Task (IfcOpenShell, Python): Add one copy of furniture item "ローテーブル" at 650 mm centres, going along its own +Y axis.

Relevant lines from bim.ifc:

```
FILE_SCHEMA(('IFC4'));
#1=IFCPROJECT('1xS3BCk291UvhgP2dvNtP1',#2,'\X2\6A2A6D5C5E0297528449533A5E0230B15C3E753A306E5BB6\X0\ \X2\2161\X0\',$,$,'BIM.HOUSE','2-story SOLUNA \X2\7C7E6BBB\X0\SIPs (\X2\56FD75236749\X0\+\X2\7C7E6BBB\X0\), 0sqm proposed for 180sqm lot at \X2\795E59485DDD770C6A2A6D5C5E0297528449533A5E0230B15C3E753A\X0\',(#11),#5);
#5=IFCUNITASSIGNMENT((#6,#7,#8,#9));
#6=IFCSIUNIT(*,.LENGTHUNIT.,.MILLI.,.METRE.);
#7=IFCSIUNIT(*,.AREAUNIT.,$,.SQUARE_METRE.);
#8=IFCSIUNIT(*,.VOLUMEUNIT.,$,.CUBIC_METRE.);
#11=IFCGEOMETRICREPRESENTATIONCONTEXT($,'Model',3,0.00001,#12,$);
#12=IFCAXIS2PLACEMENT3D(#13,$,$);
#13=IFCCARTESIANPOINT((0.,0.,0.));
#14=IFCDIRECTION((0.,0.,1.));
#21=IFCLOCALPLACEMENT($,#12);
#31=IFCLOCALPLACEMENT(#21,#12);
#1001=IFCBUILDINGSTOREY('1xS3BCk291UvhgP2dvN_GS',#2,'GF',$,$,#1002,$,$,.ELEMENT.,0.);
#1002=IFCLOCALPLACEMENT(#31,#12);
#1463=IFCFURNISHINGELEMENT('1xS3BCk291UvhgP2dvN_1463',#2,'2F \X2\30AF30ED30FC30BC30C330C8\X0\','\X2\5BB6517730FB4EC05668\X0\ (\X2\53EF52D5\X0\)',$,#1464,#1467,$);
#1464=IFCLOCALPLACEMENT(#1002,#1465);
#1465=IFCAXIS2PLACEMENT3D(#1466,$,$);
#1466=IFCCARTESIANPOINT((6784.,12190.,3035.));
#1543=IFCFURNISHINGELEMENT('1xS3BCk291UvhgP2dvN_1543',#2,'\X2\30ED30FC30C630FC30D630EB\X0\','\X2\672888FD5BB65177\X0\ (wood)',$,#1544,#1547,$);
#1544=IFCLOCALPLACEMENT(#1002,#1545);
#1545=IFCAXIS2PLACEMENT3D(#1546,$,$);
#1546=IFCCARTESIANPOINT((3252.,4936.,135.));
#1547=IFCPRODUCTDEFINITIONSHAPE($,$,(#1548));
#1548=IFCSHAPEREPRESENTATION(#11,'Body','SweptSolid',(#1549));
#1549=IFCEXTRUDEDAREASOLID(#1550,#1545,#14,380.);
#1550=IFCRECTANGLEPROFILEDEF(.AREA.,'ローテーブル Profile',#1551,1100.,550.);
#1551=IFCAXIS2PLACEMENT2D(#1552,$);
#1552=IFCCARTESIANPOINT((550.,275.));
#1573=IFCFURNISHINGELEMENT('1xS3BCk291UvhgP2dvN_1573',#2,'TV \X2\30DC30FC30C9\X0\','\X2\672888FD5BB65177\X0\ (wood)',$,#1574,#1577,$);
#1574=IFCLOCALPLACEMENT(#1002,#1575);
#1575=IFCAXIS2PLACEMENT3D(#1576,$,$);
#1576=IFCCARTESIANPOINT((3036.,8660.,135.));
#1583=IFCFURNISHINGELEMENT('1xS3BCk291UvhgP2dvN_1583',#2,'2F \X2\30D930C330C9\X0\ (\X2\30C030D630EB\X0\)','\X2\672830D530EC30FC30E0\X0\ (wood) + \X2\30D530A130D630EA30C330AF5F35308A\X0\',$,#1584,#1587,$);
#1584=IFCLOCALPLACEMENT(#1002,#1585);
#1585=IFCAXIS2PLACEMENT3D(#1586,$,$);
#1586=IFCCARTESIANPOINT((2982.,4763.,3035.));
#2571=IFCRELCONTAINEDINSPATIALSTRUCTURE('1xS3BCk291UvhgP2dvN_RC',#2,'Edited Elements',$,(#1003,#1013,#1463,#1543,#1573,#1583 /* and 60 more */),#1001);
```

```python
import ifcopenshell
import ifcopenshell.api.geometry
import ifcopenshell.api.root
import ifcopenshell.util.element
import ifcopenshell.util.placement
import ifcopenshell.util.unit

model = ifcopenshell.open("bim.ifc")
unit_scale = ifcopenshell.util.unit.calculate_unit_scale(model)


def reuse_history(source, copy):
    """copy_class also copies each property set's owner history, people and application; keep the originals."""
    for rel in copy.IsDefinedBy:
        if rel.is_a("IfcRelDefinesByProperties") and (history := rel.RelatingPropertyDefinition.OwnerHistory):
            rel.RelatingPropertyDefinition.OwnerHistory = source.OwnerHistory
            ifcopenshell.util.element.remove_deep2(model, history)


source = model.by_guid("1xS3BCk291UvhgP2dvN_1543")
base = ifcopenshell.util.placement.get_local_placement(source.ObjectPlacement)
step = base[:3, 1] * 0.65 / unit_scale

for i in range(1, 2):
    copy = ifcopenshell.api.root.copy_class(model, product=source)
    copy.Representation = ifcopenshell.util.element.copy_deep(
        model, source.Representation, exclude=["IfcGeometricRepresentationContext", "IfcRepresentationMap"]
    )
    reuse_history(source, copy)
    matrix = base.copy()
    matrix[:3, 3] += i * step
    print("added at", matrix[:3, 3].round(3) + 0.0)
    ifcopenshell.api.geometry.edit_object_placement(model, product=copy, matrix=matrix, is_si=False)

model.write("bim-out.ifc")
```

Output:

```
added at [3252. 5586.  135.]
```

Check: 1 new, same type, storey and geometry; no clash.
